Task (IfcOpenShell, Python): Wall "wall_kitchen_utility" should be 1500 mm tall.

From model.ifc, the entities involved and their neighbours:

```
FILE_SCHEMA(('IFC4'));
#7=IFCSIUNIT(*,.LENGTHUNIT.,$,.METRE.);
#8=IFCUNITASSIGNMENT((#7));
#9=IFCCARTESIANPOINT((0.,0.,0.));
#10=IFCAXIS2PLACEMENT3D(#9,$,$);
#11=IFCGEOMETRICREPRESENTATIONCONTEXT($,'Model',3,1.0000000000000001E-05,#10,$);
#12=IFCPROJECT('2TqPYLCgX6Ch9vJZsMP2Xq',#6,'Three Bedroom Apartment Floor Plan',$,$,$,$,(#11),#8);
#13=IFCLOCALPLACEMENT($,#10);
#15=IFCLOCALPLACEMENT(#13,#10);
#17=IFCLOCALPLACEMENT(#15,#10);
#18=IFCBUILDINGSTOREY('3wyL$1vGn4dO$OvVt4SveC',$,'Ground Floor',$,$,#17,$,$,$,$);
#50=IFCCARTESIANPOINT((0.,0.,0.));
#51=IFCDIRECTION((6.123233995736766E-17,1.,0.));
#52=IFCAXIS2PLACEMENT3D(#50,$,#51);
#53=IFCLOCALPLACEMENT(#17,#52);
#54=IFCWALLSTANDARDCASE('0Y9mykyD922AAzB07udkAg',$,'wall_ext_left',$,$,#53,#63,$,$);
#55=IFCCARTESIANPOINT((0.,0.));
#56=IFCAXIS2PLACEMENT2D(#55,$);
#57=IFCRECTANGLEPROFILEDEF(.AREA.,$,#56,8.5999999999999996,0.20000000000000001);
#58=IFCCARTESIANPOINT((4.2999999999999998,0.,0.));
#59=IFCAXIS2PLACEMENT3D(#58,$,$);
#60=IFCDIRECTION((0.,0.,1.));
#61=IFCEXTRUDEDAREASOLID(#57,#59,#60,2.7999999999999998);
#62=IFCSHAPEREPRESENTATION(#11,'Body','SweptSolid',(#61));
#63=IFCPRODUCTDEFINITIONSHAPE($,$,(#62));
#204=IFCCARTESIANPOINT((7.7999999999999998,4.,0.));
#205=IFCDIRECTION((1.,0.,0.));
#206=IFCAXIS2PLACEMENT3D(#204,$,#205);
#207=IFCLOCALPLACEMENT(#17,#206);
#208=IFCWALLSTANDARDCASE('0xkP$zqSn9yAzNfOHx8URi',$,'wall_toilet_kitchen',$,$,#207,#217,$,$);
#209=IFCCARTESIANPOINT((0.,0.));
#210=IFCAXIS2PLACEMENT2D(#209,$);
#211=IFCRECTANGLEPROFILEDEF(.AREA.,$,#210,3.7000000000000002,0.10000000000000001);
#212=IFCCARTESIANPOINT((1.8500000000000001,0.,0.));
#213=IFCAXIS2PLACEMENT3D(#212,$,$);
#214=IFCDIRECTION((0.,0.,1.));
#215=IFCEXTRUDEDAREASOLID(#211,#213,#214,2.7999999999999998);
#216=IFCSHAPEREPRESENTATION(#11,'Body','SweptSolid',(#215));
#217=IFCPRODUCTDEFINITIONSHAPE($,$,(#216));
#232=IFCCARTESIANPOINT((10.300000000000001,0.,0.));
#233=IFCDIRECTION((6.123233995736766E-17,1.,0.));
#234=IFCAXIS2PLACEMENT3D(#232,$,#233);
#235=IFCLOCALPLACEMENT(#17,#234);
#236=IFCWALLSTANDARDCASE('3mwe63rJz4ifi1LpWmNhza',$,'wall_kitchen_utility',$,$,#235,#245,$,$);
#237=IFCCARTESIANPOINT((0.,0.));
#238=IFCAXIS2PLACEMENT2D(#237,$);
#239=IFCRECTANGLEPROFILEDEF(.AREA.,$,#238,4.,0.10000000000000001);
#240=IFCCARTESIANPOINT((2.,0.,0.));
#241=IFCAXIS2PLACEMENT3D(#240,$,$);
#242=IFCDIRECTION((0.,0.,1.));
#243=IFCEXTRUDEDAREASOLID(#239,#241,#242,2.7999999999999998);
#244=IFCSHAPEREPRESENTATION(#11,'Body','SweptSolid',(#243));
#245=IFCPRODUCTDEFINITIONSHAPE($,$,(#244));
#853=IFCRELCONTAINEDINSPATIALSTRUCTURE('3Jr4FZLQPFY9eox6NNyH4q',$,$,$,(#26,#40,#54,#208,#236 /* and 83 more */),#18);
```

```python
import ifcopenshell
import ifcopenshell.geom
import ifcopenshell.util.shape
import ifcopenshell.util.unit

model = ifcopenshell.open("model.ifc")
unit_scale = ifcopenshell.util.unit.calculate_unit_scale(model)
settings = ifcopenshell.geom.settings()


def volume(element):
    """Net volume in cubic metres, openings subtracted."""
    shape = ifcopenshell.geom.create_shape(settings, element)
    return ifcopenshell.util.shape.get_volume(shape.geometry)


wall = model.by_guid("3mwe63rJz4ifi1LpWmNhza")
before = volume(wall)

body = next(r for r in wall.Representation.Representations if r.RepresentationIdentifier == "Body")
solid = body.Items[0]
old_height = solid.Depth
solid.Depth = 1.5 / unit_scale
after = volume(wall)

print(f"height {old_height:g} -> {solid.Depth:g}, volume {before:.3f} -> {after:.3f} m3")

model.write("model_rev.ifc")
```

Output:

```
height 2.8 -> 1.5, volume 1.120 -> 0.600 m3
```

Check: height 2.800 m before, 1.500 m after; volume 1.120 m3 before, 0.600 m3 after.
